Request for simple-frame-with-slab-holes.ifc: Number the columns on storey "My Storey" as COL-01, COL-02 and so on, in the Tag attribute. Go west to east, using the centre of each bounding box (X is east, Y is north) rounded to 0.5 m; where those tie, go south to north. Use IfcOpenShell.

First a look at what the model holds.

```python
import ifcopenshell
import ifcopenshell.util.element
import ifcopenshell.util.placement

model = ifcopenshell.open("simple-frame-with-slab-holes.ifc")
print(model.schema)
storey = next(s for s in model.by_type("IfcBuildingStorey") if s.Name == "My Storey")
columns = [e for e in ifcopenshell.util.element.get_decomposition(storey) if e.is_a("IfcColumn")]
for e in sorted(columns, key=lambda e: e.id()):
    origin = ifcopenshell.util.placement.get_local_placement(e.ObjectPlacement)[:3, 3]
    print(e.id(), e.Tag, e.Name, origin.round(2) + 0.0, sep=" | ")
```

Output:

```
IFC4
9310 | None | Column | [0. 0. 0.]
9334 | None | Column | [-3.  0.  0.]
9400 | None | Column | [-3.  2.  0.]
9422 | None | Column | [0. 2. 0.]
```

```python
import ifcopenshell
import ifcopenshell.geom
import ifcopenshell.util.element
import ifcopenshell.util.shape

model = ifcopenshell.open("simple-frame-with-slab-holes.ifc")
settings = ifcopenshell.geom.settings()
settings.set("use-world-coords", True)


def centre(element):
    shape = ifcopenshell.geom.create_shape(settings, element)
    return ifcopenshell.util.shape.get_bbox_centroid(shape.geometry)


storey = next(s for s in model.by_type("IfcBuildingStorey") if s.Name == "My Storey")
columns = [e for e in ifcopenshell.util.element.get_decomposition(storey) if e.is_a("IfcColumn")]

# Insertion points can sit at a corner or the storey origin, so sort by the geometry (in metres).
centres = {e: centre(e) for e in columns}
columns.sort(key=lambda e: (round(centres[e][0] / 0.5), centres[e][1]))

for i, e in enumerate(columns, start=1):
    number = f"COL-{i:02d}"
    e.Tag = number
    print(e.id(), number)

model.write("simple-frame-with-slab-holes_updated.ifc")
```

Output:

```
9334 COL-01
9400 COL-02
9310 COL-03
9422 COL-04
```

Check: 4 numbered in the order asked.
